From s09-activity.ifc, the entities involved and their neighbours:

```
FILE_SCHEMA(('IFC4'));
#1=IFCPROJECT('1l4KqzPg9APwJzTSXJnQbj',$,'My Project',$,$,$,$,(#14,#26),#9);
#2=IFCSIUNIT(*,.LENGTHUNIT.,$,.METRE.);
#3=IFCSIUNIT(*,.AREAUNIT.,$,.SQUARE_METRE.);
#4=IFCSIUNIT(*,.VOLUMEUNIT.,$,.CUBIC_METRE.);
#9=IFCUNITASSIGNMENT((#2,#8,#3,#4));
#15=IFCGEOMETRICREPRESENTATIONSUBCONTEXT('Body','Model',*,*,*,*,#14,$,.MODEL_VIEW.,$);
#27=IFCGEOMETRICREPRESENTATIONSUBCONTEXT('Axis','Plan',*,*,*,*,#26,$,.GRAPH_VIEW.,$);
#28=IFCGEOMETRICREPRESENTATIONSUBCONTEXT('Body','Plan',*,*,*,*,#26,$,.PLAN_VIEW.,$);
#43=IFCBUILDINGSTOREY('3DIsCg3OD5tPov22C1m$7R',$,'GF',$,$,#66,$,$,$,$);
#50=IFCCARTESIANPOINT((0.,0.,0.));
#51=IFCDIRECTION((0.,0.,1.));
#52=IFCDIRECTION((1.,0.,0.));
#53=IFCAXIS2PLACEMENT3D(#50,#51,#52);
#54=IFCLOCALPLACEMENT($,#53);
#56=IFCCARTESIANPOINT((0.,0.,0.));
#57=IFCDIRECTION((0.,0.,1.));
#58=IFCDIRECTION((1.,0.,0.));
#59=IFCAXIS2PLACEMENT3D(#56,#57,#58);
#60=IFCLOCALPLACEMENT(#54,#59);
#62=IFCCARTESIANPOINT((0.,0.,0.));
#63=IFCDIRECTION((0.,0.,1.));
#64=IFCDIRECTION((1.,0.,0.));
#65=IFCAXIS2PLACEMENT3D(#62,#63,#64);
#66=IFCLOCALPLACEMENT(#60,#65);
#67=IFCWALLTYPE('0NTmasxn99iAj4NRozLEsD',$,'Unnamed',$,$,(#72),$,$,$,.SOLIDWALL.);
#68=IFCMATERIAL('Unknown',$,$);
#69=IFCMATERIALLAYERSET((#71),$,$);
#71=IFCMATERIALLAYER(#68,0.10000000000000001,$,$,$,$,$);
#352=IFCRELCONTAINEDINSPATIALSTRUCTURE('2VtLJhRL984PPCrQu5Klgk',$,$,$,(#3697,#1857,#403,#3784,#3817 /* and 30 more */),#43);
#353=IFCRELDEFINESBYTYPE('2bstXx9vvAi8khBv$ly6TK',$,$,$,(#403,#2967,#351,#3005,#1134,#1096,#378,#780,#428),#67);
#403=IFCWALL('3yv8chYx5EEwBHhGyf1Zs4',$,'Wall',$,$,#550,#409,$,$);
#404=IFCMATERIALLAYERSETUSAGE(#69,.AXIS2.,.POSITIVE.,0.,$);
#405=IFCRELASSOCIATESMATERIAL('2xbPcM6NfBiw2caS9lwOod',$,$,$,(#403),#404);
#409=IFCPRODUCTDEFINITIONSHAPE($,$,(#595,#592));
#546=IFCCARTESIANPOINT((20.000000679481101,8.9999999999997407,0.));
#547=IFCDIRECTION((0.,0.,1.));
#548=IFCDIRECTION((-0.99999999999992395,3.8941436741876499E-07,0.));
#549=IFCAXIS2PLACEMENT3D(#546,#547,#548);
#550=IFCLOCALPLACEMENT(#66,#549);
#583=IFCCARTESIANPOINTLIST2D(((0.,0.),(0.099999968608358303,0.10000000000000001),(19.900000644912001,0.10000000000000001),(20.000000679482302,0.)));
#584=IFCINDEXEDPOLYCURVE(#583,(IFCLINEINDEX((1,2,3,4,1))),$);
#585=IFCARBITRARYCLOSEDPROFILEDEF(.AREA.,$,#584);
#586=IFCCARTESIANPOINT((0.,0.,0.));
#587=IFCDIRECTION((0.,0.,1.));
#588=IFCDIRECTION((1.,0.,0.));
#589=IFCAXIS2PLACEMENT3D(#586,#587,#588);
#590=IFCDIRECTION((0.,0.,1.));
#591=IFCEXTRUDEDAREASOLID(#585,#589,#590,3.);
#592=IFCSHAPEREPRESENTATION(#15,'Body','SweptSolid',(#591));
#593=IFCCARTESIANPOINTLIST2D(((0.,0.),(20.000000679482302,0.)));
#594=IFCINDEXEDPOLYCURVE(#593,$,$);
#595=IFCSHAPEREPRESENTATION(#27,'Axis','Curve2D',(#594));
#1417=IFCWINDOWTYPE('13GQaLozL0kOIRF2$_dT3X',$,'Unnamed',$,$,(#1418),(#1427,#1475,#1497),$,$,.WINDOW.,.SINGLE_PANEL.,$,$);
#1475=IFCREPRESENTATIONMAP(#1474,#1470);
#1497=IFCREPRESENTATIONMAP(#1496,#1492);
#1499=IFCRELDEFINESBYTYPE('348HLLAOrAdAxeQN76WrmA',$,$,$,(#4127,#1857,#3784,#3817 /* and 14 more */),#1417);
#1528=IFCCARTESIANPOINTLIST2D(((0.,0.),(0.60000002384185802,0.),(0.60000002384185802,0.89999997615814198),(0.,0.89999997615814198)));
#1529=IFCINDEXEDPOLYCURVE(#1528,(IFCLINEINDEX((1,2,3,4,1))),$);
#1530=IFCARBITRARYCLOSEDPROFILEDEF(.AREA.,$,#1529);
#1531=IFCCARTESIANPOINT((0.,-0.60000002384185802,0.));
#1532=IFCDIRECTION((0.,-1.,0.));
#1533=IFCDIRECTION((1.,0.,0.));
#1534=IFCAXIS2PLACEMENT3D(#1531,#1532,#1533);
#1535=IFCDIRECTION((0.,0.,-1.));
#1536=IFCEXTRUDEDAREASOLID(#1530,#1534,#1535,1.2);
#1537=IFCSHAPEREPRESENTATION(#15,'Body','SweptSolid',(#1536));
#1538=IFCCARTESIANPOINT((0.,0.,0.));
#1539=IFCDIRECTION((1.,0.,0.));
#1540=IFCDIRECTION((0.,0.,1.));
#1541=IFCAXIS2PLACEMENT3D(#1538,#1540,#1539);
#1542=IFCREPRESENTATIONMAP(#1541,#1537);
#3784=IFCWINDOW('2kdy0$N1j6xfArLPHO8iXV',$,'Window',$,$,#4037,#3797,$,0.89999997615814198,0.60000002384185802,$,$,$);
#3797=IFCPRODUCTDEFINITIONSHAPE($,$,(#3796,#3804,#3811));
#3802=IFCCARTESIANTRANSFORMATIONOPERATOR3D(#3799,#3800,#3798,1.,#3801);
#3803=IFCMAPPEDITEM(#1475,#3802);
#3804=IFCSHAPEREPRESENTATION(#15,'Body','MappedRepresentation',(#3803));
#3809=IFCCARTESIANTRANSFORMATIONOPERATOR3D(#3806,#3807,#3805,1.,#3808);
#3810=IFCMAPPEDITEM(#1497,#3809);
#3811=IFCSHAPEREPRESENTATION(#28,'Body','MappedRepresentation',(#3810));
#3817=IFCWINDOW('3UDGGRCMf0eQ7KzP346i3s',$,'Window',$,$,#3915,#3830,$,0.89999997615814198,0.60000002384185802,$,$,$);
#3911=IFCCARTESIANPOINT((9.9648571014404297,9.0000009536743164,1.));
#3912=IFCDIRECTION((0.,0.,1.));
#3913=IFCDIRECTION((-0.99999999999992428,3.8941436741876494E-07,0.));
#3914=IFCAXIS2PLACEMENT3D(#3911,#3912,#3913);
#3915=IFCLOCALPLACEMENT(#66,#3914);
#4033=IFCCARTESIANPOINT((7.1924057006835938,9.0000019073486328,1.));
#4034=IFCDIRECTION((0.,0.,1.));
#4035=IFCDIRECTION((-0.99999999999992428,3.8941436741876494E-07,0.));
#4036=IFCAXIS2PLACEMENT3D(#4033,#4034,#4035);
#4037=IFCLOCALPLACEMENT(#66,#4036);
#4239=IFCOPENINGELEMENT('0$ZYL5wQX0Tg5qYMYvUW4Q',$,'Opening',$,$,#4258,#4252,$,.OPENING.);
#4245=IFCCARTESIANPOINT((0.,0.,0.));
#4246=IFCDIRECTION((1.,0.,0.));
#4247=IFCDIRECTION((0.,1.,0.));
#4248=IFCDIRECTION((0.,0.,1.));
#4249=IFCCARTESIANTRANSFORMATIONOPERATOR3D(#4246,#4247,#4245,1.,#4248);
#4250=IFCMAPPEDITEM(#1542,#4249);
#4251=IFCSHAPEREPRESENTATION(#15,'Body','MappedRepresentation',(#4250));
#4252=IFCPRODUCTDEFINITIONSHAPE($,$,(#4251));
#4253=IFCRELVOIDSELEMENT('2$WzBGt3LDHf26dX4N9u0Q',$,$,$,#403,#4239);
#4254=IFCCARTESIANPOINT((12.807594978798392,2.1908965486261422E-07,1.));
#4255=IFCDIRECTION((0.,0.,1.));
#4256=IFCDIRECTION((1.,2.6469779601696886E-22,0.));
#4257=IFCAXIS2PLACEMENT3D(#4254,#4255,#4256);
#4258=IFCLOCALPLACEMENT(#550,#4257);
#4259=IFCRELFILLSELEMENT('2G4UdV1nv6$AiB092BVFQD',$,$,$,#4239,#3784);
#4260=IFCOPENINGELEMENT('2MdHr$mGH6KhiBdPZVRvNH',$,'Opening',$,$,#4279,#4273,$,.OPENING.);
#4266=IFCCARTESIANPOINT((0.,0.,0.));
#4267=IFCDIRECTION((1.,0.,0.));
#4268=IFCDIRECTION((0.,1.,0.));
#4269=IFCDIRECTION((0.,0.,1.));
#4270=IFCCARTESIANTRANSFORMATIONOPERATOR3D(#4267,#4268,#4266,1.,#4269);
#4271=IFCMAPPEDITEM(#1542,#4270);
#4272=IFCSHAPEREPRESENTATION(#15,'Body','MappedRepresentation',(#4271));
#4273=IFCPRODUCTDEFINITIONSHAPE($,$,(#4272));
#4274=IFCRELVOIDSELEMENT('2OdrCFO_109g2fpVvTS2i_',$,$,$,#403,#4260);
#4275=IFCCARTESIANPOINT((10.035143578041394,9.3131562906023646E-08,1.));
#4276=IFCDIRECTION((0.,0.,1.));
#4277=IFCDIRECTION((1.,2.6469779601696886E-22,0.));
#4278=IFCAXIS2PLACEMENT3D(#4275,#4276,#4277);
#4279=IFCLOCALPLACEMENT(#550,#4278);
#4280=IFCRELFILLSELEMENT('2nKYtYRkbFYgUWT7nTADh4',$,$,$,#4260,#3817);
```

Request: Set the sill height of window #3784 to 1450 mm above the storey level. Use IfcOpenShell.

```python
import numpy as np
import ifcopenshell
import ifcopenshell.api.geometry
import ifcopenshell.geom
import ifcopenshell.util.element
import ifcopenshell.util.placement
import ifcopenshell.util.shape
import ifcopenshell.util.unit

model = ifcopenshell.open("s09-activity.ifc")
unit_scale = ifcopenshell.util.unit.calculate_unit_scale(model)

window = model.by_guid("2kdy0$N1j6xfArLPHO8iXV")
opening = window.FillsVoids[0].RelatingOpeningElement
storey = ifcopenshell.util.element.get_container(window, ifc_class="IfcBuildingStorey")
level = ifcopenshell.util.placement.get_local_placement(storey.ObjectPlacement)[2, 3]

# The opening's origin need not be at the sill, so measure its lowest point.
shape = ifcopenshell.geom.create_shape(ifcopenshell.geom.settings(), opening)
bottom = ifcopenshell.util.shape.get_shape_bottom_elevation(shape, shape.geometry) / unit_scale
dz = level + 1.45 - bottom

shift = np.array([0.0, 0.0, dz])
# The window is not placed relative to its opening, so move both.
for product in (opening, window):
    matrix = ifcopenshell.util.placement.get_local_placement(product.ObjectPlacement)
    matrix[:3, 3] += shift
    ifcopenshell.api.geometry.edit_object_placement(model, product=product, matrix=matrix, is_si=False)

print(f"moved by {dz * unit_scale:+.3f} m")

model.write("s09-activity_edited.ifc")
```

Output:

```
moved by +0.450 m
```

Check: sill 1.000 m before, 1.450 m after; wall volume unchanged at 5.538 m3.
